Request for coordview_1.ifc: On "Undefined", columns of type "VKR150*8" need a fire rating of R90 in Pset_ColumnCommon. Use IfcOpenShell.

First a look at what the model holds.

```python
import ifcopenshell
import ifcopenshell.util.element

model = ifcopenshell.open("coordview_1.ifc")
print(model.schema)
storey = next(s for s in model.by_type("IfcBuildingStorey") if s.Name == "Undefined")
columns = [e for e in ifcopenshell.util.element.get_decomposition(storey) if e.is_a("IfcColumn")]
seen = {}
for e in columns:
    element_type = ifcopenshell.util.element.get_type(e)
    key = (element_type.Name if element_type != e and element_type else None, ifcopenshell.util.element.get_pset(e, "Pset_ColumnCommon", "FireRating"))
    seen[key] = seen.get(key, 0) + 1
for (name, value), count in sorted(seen.items(), key=str):
    print(count, "x", name, "|", value)
```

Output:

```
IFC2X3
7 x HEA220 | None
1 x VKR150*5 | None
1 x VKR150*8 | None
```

```python
import ifcopenshell
import ifcopenshell.api.pset
import ifcopenshell.util.element

model = ifcopenshell.open("coordview_1.ifc")

storey = next(s for s in model.by_type("IfcBuildingStorey") if s.Name == "Undefined")
columns = [e for e in ifcopenshell.util.element.get_decomposition(storey) if e.is_a("IfcColumn")]

count = 0
for e in columns:
    element_type = ifcopenshell.util.element.get_type(e)
    if element_type in (None, e) or element_type.Name != "VKR150*8":
        continue
    found = ifcopenshell.util.element.get_pset(e, "Pset_ColumnCommon", should_inherit=False)
    if found:
        pset = model.by_id(found["id"])
        if len(ifcopenshell.util.element.get_elements_by_pset(pset)) > 1:
            pset = ifcopenshell.api.pset.unshare_pset(model, products=[e], pset=pset)[0]
    else:
        pset = ifcopenshell.api.pset.add_pset(model, product=e, name="Pset_ColumnCommon")
    ifcopenshell.api.pset.edit_pset(model, pset=pset, properties={"FireRating": "R90"})
    count += 1

print(count, "columns updated")

model.write("coordview_1-out.ifc")
```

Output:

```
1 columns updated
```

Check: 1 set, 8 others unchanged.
